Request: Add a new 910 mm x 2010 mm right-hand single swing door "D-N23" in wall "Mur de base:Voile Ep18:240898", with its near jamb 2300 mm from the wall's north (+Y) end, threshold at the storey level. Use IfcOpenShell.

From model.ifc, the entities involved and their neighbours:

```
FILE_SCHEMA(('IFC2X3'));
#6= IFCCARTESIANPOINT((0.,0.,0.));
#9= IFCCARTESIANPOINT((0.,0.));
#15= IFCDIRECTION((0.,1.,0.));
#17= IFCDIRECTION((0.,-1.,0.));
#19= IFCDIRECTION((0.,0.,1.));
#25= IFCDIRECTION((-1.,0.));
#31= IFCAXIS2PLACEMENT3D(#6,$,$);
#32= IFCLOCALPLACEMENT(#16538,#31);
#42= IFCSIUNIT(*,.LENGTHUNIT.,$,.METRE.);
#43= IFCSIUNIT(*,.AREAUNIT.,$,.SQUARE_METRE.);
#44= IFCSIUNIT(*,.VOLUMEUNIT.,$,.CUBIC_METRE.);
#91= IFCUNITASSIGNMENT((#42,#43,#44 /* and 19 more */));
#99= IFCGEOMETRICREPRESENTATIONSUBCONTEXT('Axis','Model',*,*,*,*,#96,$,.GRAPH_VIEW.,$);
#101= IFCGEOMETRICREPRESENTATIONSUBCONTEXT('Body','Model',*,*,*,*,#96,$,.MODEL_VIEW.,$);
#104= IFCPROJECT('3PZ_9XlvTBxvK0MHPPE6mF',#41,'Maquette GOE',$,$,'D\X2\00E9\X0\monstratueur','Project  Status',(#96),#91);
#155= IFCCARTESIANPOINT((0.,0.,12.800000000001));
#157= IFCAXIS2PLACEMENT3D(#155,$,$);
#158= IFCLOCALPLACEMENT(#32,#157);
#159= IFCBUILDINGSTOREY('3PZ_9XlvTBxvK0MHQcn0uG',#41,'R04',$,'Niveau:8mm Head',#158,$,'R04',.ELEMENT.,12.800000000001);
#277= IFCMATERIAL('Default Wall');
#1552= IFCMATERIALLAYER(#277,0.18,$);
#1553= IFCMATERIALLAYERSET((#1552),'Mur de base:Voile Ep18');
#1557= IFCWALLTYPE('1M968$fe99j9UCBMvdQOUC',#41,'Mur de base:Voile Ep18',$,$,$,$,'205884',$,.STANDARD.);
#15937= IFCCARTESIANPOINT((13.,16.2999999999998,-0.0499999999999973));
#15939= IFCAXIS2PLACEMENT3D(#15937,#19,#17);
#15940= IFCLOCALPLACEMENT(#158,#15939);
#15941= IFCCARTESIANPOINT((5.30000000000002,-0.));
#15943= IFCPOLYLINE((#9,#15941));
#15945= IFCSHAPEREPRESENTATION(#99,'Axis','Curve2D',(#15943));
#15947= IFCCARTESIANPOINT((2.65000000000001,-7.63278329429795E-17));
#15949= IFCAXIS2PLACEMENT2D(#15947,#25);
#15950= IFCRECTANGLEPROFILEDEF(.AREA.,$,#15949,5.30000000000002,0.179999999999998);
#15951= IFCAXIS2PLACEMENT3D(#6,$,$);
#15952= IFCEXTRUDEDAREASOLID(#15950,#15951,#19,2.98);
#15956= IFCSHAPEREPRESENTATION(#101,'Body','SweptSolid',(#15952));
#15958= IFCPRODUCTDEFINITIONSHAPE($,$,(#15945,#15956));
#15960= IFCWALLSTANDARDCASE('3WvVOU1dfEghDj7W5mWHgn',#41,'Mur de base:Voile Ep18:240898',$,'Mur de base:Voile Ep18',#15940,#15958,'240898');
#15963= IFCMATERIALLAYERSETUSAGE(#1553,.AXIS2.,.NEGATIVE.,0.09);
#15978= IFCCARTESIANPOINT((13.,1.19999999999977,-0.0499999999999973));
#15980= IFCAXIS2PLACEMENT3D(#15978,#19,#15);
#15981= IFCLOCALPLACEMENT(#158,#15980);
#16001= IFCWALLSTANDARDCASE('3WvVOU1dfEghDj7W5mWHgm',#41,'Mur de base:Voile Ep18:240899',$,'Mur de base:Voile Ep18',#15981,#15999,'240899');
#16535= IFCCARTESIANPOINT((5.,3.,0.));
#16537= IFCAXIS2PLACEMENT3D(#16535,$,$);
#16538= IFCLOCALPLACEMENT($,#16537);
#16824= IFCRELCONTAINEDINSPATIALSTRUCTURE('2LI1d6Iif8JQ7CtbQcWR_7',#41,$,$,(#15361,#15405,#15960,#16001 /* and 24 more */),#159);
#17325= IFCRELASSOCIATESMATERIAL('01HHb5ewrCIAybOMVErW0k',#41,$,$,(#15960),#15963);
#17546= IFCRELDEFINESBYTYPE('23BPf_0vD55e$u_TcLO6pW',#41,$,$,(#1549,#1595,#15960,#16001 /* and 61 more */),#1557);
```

```python
import numpy as np
import ifcopenshell
import ifcopenshell.api.feature
import ifcopenshell.api.geometry
import ifcopenshell.api.root
import ifcopenshell.api.spatial
import ifcopenshell.api.type
import ifcopenshell.geom
import ifcopenshell.util.element
import ifcopenshell.util.placement
import ifcopenshell.util.representation
import ifcopenshell.util.shape
import ifcopenshell.util.unit

model = ifcopenshell.open("model.ifc")
unit_scale = ifcopenshell.util.unit.calculate_unit_scale(model)
settings = ifcopenshell.geom.settings()


def volume(element):
    """Net volume in cubic metres, openings subtracted."""
    shape = ifcopenshell.geom.create_shape(settings, element)
    return ifcopenshell.util.shape.get_volume(shape.geometry)


wall = model.by_guid("3WvVOU1dfEghDj7W5mWHgn")
storey = ifcopenshell.util.element.get_container(wall, ifc_class="IfcBuildingStorey")
context = ifcopenshell.util.representation.get_context(model, "Model", "Body", "MODEL_VIEW")
before = volume(wall)

width, height, from_end, sill = 0.91, 2.01, 2.3, 0.0  # metres

# The wall runs along its own X axis, and the end named is its -X end.
wall_shape = ifcopenshell.geom.create_shape(settings, wall)
x, y, z = ifcopenshell.util.shape.get_vertices(wall_shape.geometry).T
start = x.min() + from_end
face, thickness = float(y.min()), float(y.max() - y.min())
wall_matrix = ifcopenshell.util.placement.get_local_placement(wall.ObjectPlacement)
level = ifcopenshell.util.placement.get_local_placement(storey.ObjectPlacement)[2, 3]


def in_wall(x, y):
    """Placement at x, y metres in the wall's axes, at sill height."""
    matrix = wall_matrix.copy()
    matrix[:, 3] = wall_matrix @ np.array([x / unit_scale, y / unit_scale, 0.0, 1.0])
    matrix[2, 3] = level + sill / unit_scale
    return matrix


# Opening: a box that overshoots both wall faces by 50 mm.
opening = ifcopenshell.api.root.create_entity(model, ifc_class="IfcOpeningElement")
box = ifcopenshell.api.geometry.add_wall_representation(
    model, context=context, length=width, height=height, thickness=thickness + 0.1
)
ifcopenshell.api.geometry.assign_representation(model, product=opening, representation=box)
ifcopenshell.api.geometry.edit_object_placement(model, product=opening, matrix=in_wall(start, face - 0.05), is_si=False)
ifcopenshell.api.feature.add_feature(model, feature=opening, element=wall)

door = ifcopenshell.api.root.create_entity(model, ifc_class="IfcDoor", name="D-N23")
door.OverallWidth, door.OverallHeight = width / unit_scale, height / unit_scale
body = ifcopenshell.api.geometry.add_door_representation(
    model,
    context=context,
    overall_width=door.OverallWidth,
    overall_height=door.OverallHeight,
    operation_type="SINGLE_SWING_RIGHT",
    lining_properties={"LiningDepth": thickness / unit_scale, "ThresholdDepth": thickness / unit_scale},
)
ifcopenshell.api.geometry.assign_representation(model, product=door, representation=body)
ifcopenshell.api.spatial.assign_container(model, products=[door], relating_structure=storey)
fills = ifcopenshell.api.feature.add_filling(model, opening=opening, element=door)
fills.OwnerHistory = door.OwnerHistory  # required in IFC2X3

# IFC2X3 keeps the operation on the door style.
style = ifcopenshell.api.root.create_entity(model, ifc_class="IfcDoorStyle", name="D-N23")
style.OperationType, style.ConstructionType = "SINGLE_SWING_RIGHT", "NOTDEFINED"
style.ParameterTakesPrecedence = style.Sizeable = False
ifcopenshell.api.type.assign_type(model, related_objects=[door], relating_type=style)

# The lining spans the wall, so the door starts at the wall face.
ifcopenshell.api.geometry.edit_object_placement(model, product=door, matrix=in_wall(start, face), is_si=False)

after = volume(wall)

print(f"wall volume {before:.3f} -> {after:.3f} m3")

model.write("model_edited.ifc")
```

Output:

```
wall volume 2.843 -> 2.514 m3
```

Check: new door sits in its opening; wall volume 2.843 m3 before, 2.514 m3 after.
